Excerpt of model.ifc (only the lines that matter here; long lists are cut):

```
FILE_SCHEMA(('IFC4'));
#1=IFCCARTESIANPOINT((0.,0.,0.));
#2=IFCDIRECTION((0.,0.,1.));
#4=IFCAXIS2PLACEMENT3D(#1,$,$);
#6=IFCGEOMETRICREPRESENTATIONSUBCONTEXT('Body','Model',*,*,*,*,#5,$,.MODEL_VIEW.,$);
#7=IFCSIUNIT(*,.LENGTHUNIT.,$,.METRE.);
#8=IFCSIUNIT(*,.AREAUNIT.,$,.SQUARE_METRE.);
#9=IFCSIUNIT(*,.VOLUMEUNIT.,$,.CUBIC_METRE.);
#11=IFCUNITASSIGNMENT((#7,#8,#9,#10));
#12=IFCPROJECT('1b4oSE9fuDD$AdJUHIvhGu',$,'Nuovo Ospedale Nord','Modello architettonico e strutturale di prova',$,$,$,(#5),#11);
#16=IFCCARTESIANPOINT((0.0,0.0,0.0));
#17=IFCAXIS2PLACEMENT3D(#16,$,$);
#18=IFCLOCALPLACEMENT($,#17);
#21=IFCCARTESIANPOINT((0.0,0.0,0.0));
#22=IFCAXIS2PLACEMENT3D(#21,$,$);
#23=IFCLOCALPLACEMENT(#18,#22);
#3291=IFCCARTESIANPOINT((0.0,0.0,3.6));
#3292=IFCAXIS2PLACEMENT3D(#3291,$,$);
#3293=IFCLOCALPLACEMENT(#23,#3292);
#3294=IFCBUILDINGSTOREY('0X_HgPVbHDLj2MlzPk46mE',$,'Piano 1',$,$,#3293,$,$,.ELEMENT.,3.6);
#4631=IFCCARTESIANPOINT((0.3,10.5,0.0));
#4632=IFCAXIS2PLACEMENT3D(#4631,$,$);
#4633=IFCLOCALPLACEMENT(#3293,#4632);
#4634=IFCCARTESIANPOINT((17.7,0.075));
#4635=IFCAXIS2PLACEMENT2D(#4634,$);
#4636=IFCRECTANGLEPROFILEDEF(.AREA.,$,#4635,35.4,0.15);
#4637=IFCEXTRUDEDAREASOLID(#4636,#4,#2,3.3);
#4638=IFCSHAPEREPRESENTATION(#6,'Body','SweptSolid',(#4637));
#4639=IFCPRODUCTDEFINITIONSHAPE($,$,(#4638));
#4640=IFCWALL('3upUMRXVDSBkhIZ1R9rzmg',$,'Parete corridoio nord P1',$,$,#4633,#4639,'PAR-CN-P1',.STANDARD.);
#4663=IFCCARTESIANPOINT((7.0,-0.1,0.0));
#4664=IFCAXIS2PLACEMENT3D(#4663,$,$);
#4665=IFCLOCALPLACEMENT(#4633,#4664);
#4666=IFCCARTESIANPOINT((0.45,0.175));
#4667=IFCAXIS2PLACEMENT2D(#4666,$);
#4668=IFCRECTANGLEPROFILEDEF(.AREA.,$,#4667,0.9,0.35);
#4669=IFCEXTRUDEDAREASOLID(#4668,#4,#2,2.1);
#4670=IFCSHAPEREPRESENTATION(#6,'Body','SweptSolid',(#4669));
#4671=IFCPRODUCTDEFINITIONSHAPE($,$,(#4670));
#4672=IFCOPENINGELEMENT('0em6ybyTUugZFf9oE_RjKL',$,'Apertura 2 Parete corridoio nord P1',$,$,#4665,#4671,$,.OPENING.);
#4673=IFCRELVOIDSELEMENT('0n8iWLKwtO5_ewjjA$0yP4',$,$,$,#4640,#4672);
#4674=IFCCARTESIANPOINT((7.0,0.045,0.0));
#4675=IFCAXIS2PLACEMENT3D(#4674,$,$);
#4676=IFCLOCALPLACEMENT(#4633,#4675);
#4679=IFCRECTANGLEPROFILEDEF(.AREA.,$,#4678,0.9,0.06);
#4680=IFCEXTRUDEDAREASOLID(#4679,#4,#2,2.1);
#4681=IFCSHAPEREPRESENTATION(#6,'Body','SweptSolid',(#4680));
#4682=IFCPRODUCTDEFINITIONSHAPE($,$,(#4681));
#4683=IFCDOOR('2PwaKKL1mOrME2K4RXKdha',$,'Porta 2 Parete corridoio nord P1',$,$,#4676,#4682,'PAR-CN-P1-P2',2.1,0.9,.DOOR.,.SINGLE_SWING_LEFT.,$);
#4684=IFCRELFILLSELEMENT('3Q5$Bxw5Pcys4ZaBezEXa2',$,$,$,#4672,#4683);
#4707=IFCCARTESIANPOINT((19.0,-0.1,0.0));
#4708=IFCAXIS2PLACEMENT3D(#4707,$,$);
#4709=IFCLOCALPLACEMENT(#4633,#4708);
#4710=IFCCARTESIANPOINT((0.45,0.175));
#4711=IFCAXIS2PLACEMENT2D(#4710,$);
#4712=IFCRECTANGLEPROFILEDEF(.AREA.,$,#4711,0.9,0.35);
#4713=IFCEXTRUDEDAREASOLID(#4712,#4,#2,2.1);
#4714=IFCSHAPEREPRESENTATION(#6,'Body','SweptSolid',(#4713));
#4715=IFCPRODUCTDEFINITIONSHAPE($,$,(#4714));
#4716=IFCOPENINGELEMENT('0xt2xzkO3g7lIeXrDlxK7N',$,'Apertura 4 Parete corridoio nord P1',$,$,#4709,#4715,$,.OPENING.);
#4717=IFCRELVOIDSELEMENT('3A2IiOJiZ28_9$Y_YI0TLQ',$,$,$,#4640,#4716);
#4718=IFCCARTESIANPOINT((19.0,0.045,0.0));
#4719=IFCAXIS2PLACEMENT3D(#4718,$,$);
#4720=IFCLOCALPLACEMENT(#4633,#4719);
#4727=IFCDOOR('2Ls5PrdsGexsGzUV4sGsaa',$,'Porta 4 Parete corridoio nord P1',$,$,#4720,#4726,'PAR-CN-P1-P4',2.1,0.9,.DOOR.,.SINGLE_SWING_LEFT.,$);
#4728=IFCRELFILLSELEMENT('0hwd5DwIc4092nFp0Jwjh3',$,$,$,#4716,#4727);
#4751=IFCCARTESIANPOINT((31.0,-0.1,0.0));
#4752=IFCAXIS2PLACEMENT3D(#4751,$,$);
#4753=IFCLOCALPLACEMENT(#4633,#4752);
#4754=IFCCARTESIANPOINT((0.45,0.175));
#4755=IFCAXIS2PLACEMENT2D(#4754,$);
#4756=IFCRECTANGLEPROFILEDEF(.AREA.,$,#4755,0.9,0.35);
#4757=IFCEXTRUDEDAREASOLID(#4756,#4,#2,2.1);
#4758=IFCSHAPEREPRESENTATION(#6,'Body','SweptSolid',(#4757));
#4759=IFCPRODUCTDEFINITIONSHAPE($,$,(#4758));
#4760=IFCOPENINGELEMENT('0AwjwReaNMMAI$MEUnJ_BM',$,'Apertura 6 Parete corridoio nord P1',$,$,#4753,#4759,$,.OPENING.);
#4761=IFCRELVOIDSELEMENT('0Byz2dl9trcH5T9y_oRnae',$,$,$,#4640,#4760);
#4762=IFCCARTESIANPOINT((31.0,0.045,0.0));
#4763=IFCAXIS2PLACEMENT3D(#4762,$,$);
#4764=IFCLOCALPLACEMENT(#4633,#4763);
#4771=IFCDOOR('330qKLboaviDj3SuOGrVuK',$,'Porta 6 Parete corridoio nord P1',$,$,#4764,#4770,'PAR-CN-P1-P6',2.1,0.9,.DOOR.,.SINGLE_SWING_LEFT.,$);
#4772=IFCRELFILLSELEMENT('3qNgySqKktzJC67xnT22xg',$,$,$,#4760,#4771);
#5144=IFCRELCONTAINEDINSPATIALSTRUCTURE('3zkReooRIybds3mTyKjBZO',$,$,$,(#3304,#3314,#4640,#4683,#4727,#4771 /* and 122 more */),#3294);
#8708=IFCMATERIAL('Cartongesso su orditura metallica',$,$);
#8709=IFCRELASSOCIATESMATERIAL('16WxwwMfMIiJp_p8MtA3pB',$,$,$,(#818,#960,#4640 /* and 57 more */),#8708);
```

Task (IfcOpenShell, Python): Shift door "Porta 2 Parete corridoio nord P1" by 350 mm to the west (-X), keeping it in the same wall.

```python
import ifcopenshell
import ifcopenshell.api.geometry
import ifcopenshell.util.placement

model = ifcopenshell.open("model.ifc")

door = model.by_id(4683)
opening = door.FillsVoids[0].RelatingOpeningElement
wall = opening.VoidsElements[0].RelatingBuildingElement

wall_matrix = ifcopenshell.util.placement.get_local_placement(wall.ObjectPlacement)
shift = wall_matrix[:3, 0] * -0.35
before = ifcopenshell.util.placement.get_local_placement(door.ObjectPlacement)[:3, 3].copy()

# The door is not placed relative to its opening, so move both.
for product in (opening, door):
    matrix = ifcopenshell.util.placement.get_local_placement(product.ObjectPlacement)
    matrix[:3, 3] += shift
    ifcopenshell.api.geometry.edit_object_placement(model, product=product, matrix=matrix, is_si=False)

after = ifcopenshell.util.placement.get_local_placement(door.ObjectPlacement)[:3, 3]
print("door moved by", (after - before).round(3) + 0.0)

model.write("model_edited.ifc")
```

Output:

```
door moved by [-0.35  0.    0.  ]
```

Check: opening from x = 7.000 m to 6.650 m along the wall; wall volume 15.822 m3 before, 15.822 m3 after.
